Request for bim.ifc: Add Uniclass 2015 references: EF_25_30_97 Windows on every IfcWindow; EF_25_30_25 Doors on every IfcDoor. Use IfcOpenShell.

First a look at what the model holds.

```python
import ifcopenshell

model = ifcopenshell.open("bim.ifc")
print(model.schema)
print("classifications:", [c.Name for c in model.by_type("IfcClassification")])
for ifc_class in ("IfcDoor", "IfcRoof", "IfcStair", "IfcWall", "IfcWindow"):
    print(ifc_class, len(model.by_type(ifc_class)))
```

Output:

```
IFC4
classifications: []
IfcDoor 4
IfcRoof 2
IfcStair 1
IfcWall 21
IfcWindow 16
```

```python
import ifcopenshell
import ifcopenshell.api.classification

model = ifcopenshell.open("bim.ifc")

system = ifcopenshell.api.classification.add_classification(model, classification="Uniclass 2015")

codes = {
    "IfcWindow": ("EF_25_30_97", "Windows"),
    "IfcDoor": ("EF_25_30_25", "Doors"),
}
for ifc_class, (code, name) in codes.items():
    products = model.by_type(ifc_class)
    ifcopenshell.api.classification.add_reference(
        model, products=products, classification=system, identification=code, name=name
    )
    print(code, len(products))

model.write("bim_edited.ifc")
```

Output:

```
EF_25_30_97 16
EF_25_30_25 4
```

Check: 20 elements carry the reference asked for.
